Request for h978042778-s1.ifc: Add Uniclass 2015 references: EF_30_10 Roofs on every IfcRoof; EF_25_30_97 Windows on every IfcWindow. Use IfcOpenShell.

First a look at what the model holds.

```python
import ifcopenshell

model = ifcopenshell.open("h978042778-s1.ifc")
print(model.schema)
print("classifications:", [c.Name for c in model.by_type("IfcClassification")])
for ifc_class in ("IfcDoor", "IfcRoof", "IfcStair", "IfcWall", "IfcWindow"):
    print(ifc_class, len(model.by_type(ifc_class)))
```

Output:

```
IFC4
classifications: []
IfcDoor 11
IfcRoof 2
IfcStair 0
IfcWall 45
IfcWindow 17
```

```python
import ifcopenshell
import ifcopenshell.api.classification

model = ifcopenshell.open("h978042778-s1.ifc")

system = ifcopenshell.api.classification.add_classification(model, classification="Uniclass 2015")

codes = {
    "IfcRoof": ("EF_30_10", "Roofs"),
    "IfcWindow": ("EF_25_30_97", "Windows"),
}
for ifc_class, (code, name) in codes.items():
    products = model.by_type(ifc_class)
    ifcopenshell.api.classification.add_reference(
        model, products=products, classification=system, identification=code, name=name
    )
    print(code, len(products))

model.write("h978042778-s1-out.ifc")
```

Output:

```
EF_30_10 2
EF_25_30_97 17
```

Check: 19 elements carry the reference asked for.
